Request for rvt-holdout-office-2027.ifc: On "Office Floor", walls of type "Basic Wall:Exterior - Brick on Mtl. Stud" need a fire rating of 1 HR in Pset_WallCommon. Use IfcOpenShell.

First a look at what the model holds.

```python
import ifcopenshell
import ifcopenshell.util.element

model = ifcopenshell.open("rvt-holdout-office-2027.ifc")
print(model.schema)
storey = next(s for s in model.by_type("IfcBuildingStorey") if s.Name == "Office Floor")
walls = [e for e in ifcopenshell.util.element.get_decomposition(storey) if e.is_a("IfcWall")]
seen = {}
for e in walls:
    element_type = ifcopenshell.util.element.get_type(e)
    key = (element_type.Name if element_type != e and element_type else None, ifcopenshell.util.element.get_pset(e, "Pset_WallCommon", "FireRating"))
    seen[key] = seen.get(key, 0) + 1
for (name, value), count in sorted(seen.items(), key=str):
    print(count, "x", name, "|", value)
```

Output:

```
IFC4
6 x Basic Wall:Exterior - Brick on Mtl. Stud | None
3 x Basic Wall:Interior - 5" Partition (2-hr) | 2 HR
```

```python
import ifcopenshell
import ifcopenshell.api.pset
import ifcopenshell.util.element

model = ifcopenshell.open("rvt-holdout-office-2027.ifc")

storey = next(s for s in model.by_type("IfcBuildingStorey") if s.Name == "Office Floor")
walls = [e for e in ifcopenshell.util.element.get_decomposition(storey) if e.is_a("IfcWall")]

count = 0
for e in walls:
    element_type = ifcopenshell.util.element.get_type(e)
    if element_type in (None, e) or element_type.Name != "Basic Wall:Exterior - Brick on Mtl. Stud":
        continue
    # add_pset returns the element's existing set when there is one.
    pset = ifcopenshell.api.pset.add_pset(model, product=e, name="Pset_WallCommon")
    ifcopenshell.api.pset.edit_pset(model, pset=pset, properties={"FireRating": "1 HR"})
    count += 1

print(count, "walls updated")

model.write("rvt-holdout-office-2027_v2.ifc")
```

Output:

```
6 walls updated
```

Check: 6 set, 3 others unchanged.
